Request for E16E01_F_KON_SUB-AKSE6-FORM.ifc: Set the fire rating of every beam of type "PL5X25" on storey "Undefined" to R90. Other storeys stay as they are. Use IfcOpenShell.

First a look at what the model holds.

```python
import ifcopenshell
import ifcopenshell.util.element

model = ifcopenshell.open("E16E01_F_KON_SUB-AKSE6-FORM.ifc")
print(model.schema)
storey = next(s for s in model.by_type("IfcBuildingStorey") if s.Name == "Undefined")
beams = [e for e in ifcopenshell.util.element.get_decomposition(storey) if e.is_a("IfcBeam")]
seen = {}
for e in beams:
    element_type = ifcopenshell.util.element.get_type(e)
    key = (element_type.Name if element_type != e and element_type else None, ifcopenshell.util.element.get_pset(e, "Pset_BeamCommon", "FireRating"))
    seen[key] = seen.get(key, 0) + 1
for (name, value), count in sorted(seen.items(), key=str):
    print(count, "x", name, "|", value)
```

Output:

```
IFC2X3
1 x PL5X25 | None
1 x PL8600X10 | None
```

```python
import ifcopenshell
import ifcopenshell.api.pset
import ifcopenshell.util.element

model = ifcopenshell.open("E16E01_F_KON_SUB-AKSE6-FORM.ifc")

storey = next(s for s in model.by_type("IfcBuildingStorey") if s.Name == "Undefined")
beams = [e for e in ifcopenshell.util.element.get_decomposition(storey) if e.is_a("IfcBeam")]

count = 0
for e in beams:
    element_type = ifcopenshell.util.element.get_type(e)
    if element_type in (None, e) or element_type.Name != "PL5X25":
        continue
    # add_pset returns the element's existing set when there is one.
    pset = ifcopenshell.api.pset.add_pset(model, product=e, name="Pset_BeamCommon")
    ifcopenshell.api.pset.edit_pset(model, pset=pset, properties={"FireRating": "R90"})
    count += 1

print(count, "beams updated")

model.write("E16E01_F_KON_SUB-AKSE6-FORM_rev.ifc")
```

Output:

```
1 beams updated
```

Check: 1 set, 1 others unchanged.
